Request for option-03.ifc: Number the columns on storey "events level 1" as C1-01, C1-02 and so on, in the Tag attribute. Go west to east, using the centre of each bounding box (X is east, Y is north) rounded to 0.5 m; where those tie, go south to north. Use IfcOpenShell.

First a look at what the model holds.

```python
import ifcopenshell
import ifcopenshell.util.element
import ifcopenshell.util.placement

model = ifcopenshell.open("option-03.ifc")
print(model.schema)
storey = next(s for s in model.by_type("IfcBuildingStorey") if s.Name == "events level 1")
columns = [e for e in ifcopenshell.util.element.get_decomposition(storey) if e.is_a("IfcColumn")]
for e in sorted(columns, key=lambda e: e.id()):
    origin = ifcopenshell.util.placement.get_local_placement(e.ObjectPlacement)[:3, 3]
    print(e.id(), e.Tag, e.Name, origin.round(2) + 0.0, sep=" | ")
```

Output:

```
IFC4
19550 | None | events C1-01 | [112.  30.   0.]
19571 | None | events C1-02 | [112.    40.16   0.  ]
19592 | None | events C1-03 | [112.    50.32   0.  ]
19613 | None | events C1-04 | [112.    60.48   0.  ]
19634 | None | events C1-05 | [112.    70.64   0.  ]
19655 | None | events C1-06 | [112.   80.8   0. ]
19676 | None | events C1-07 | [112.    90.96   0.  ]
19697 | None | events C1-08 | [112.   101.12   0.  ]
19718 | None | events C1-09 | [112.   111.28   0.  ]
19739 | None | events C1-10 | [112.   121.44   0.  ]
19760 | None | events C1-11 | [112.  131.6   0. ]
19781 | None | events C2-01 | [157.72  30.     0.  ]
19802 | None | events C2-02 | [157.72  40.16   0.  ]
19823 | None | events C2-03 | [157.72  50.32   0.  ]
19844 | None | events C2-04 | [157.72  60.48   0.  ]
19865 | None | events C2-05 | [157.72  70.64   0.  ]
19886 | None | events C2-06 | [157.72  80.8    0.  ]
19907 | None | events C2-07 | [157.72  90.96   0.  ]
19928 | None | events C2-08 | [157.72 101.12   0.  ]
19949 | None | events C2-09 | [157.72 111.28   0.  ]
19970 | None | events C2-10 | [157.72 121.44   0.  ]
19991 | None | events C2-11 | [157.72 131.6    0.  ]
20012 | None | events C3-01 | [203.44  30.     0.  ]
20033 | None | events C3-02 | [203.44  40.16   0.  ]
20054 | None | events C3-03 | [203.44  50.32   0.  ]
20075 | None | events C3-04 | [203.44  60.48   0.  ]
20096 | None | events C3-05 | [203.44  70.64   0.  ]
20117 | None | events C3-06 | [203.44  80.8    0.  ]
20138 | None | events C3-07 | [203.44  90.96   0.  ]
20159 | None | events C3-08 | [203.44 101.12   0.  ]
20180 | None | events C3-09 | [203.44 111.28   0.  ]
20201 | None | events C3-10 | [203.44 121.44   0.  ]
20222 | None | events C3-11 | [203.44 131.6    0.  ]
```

```python
import ifcopenshell
import ifcopenshell.geom
import ifcopenshell.util.element
import ifcopenshell.util.shape

model = ifcopenshell.open("option-03.ifc")
settings = ifcopenshell.geom.settings()
settings.set("use-world-coords", True)


def centre(element):
    shape = ifcopenshell.geom.create_shape(settings, element)
    return ifcopenshell.util.shape.get_bbox_centroid(shape.geometry)


storey = next(s for s in model.by_type("IfcBuildingStorey") if s.Name == "events level 1")
columns = [e for e in ifcopenshell.util.element.get_decomposition(storey) if e.is_a("IfcColumn")]

# Insertion points can sit at a corner or the storey origin, so sort by the geometry (in metres).
centres = {e: centre(e) for e in columns}
columns.sort(key=lambda e: (round(centres[e][0] / 0.5), centres[e][1]))

for i, e in enumerate(columns, start=1):
    number = f"C1-{i:02d}"
    e.Tag = number
    print(e.id(), number)

model.write("option-03_v2.ifc")
```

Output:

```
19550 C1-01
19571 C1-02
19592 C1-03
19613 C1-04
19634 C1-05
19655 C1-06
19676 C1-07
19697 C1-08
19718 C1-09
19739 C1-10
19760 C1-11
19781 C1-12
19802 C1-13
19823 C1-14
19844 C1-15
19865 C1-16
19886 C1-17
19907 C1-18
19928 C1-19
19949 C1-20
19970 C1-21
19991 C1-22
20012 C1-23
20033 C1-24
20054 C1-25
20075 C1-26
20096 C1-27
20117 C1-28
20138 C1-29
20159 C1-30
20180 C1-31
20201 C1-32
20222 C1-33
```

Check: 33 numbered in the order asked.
